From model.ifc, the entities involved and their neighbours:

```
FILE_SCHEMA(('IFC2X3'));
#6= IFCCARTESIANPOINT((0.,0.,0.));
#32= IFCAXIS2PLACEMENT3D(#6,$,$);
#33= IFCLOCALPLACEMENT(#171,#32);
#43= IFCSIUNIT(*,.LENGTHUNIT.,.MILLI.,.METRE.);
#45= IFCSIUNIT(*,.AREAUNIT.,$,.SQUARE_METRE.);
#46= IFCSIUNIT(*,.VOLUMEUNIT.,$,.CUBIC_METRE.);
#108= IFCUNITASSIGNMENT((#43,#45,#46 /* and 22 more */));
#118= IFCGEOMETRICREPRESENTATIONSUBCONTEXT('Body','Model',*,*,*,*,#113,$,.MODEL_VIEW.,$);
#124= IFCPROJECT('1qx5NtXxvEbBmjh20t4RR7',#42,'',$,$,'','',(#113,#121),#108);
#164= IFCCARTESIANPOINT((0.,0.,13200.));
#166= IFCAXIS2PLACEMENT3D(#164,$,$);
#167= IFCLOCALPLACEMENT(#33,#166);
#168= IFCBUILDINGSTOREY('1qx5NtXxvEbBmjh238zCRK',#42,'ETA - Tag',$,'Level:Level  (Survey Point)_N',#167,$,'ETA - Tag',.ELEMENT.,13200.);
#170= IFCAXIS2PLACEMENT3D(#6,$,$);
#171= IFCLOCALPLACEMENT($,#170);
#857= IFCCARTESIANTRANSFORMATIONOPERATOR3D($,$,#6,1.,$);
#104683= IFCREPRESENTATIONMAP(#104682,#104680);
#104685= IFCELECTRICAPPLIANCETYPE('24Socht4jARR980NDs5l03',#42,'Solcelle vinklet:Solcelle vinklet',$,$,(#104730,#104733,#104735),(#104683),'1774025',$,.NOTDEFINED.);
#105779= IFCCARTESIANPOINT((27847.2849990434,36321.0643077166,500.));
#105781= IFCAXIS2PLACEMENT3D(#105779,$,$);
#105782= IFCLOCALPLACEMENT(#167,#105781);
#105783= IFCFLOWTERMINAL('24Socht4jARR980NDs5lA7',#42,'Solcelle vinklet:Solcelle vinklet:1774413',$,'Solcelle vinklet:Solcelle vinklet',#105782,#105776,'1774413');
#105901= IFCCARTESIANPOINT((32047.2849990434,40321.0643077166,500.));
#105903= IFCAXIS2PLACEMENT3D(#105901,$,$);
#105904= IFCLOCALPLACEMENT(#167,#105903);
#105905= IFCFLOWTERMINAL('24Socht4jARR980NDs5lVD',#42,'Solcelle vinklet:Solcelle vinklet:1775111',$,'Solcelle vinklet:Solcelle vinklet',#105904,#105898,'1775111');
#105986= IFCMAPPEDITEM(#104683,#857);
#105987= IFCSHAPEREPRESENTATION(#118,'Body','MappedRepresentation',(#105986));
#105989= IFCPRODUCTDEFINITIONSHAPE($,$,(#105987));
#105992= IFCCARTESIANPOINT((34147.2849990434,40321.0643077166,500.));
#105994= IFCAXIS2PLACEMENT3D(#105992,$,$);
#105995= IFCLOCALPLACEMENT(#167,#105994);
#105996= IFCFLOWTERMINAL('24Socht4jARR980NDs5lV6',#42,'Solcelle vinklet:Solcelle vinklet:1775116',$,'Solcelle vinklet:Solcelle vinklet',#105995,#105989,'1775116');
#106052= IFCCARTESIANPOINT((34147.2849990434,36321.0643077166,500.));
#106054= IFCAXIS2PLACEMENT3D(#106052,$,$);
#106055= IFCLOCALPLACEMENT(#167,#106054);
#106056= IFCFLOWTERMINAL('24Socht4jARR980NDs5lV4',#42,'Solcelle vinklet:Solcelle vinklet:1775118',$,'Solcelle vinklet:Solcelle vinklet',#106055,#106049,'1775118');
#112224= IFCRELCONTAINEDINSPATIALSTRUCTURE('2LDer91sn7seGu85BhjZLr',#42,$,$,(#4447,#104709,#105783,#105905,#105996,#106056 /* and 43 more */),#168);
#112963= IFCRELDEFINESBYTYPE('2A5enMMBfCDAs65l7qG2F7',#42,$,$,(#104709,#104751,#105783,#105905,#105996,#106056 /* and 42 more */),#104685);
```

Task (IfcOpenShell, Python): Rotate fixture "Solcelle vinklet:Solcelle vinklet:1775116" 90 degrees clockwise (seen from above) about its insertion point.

```python
import ifcopenshell
import ifcopenshell.api.geometry
import ifcopenshell.util.placement

model = ifcopenshell.open("model.ifc")

item = model.by_guid("24Socht4jARR980NDs5lV6")
matrix = ifcopenshell.util.placement.get_local_placement(item.ObjectPlacement)
matrix = matrix @ ifcopenshell.util.placement.rotation(-90, "Z")
ifcopenshell.api.geometry.edit_object_placement(model, product=item, matrix=matrix, is_si=False)

print(ifcopenshell.util.placement.get_local_placement(item.ObjectPlacement).round(3) + 0.0)

model.write("model_v2.ifc")
```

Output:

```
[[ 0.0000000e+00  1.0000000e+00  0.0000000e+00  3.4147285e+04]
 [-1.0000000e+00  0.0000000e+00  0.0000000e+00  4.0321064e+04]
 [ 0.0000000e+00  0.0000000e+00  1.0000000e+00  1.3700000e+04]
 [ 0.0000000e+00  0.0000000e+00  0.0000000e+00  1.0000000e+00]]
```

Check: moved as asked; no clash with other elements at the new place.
